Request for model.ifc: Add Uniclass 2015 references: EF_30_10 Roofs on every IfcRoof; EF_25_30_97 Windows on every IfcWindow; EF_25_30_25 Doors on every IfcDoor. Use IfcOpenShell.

First a look at what the model holds.

```python
import ifcopenshell

model = ifcopenshell.open("model.ifc")
print(model.schema)
print("classifications:", [c.Name for c in model.by_type("IfcClassification")])
for ifc_class in ("IfcDoor", "IfcRoof", "IfcStair", "IfcWall", "IfcWindow"):
    print(ifc_class, len(model.by_type(ifc_class)))
```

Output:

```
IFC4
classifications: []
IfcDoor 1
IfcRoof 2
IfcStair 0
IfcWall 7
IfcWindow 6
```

```python
import ifcopenshell
import ifcopenshell.api.classification

model = ifcopenshell.open("model.ifc")

system = ifcopenshell.api.classification.add_classification(model, classification="Uniclass 2015")

codes = {
    "IfcRoof": ("EF_30_10", "Roofs"),
    "IfcWindow": ("EF_25_30_97", "Windows"),
    "IfcDoor": ("EF_25_30_25", "Doors"),
}
for ifc_class, (code, name) in codes.items():
    products = model.by_type(ifc_class)
    ifcopenshell.api.classification.add_reference(
        model, products=products, classification=system, identification=code, name=name
    )
    print(code, len(products))

model.write("model_updated.ifc")
```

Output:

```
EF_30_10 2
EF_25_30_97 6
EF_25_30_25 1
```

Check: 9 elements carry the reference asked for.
